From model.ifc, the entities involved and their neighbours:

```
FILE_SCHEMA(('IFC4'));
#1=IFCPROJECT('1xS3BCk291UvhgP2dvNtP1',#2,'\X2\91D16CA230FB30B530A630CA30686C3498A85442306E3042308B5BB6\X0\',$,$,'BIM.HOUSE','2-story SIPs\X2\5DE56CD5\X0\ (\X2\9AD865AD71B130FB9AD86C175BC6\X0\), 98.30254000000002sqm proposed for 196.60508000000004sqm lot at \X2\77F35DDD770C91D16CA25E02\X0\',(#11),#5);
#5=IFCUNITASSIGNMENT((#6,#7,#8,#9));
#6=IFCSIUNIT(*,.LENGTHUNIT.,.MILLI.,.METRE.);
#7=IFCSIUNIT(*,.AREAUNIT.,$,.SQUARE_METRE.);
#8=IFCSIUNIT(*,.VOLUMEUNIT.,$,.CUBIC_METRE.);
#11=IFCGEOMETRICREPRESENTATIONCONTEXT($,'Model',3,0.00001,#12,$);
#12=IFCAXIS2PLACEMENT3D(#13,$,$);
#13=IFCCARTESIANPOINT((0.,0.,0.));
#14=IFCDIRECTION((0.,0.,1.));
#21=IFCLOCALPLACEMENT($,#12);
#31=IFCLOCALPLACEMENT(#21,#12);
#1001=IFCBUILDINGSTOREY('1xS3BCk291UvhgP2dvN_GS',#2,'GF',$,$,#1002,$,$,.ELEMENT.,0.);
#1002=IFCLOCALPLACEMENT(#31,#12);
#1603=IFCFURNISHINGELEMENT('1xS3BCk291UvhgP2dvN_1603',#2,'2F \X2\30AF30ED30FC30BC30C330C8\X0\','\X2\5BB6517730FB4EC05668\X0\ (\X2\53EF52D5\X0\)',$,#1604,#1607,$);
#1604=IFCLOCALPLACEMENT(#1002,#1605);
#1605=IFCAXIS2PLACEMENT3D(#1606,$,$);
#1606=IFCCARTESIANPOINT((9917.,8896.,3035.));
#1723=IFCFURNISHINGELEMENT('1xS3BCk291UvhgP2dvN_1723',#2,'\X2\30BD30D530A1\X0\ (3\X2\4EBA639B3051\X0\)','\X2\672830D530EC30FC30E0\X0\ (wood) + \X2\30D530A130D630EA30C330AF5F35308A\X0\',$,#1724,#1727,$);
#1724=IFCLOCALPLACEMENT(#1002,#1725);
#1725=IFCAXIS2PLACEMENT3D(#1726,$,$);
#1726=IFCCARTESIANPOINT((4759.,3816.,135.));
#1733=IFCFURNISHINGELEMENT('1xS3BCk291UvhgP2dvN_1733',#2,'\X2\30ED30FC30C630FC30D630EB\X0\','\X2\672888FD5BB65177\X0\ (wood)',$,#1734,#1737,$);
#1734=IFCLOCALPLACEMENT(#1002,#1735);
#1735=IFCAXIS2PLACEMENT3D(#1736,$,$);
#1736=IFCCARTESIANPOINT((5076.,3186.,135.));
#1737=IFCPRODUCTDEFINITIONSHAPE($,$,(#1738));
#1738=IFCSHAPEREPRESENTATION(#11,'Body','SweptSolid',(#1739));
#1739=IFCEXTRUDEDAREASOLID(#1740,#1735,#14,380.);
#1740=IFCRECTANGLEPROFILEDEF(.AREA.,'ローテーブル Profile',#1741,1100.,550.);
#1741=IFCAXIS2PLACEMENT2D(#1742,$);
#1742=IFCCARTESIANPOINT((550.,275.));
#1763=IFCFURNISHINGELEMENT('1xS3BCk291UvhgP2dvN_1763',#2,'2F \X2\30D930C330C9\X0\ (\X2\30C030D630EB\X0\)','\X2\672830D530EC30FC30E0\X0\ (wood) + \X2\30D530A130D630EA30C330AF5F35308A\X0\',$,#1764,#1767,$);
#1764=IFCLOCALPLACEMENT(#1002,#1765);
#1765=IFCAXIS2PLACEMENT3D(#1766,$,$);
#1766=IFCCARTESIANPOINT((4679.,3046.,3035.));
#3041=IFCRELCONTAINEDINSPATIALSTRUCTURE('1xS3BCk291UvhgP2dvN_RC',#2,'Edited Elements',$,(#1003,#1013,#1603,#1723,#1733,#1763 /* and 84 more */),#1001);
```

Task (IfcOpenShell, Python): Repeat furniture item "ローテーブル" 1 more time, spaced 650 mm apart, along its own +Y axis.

```python
import ifcopenshell
import ifcopenshell.api.geometry
import ifcopenshell.api.root
import ifcopenshell.util.element
import ifcopenshell.util.placement
import ifcopenshell.util.unit

model = ifcopenshell.open("model.ifc")
unit_scale = ifcopenshell.util.unit.calculate_unit_scale(model)


def reuse_history(source, copy):
    """copy_class also copies each property set's owner history, people and application; keep the originals."""
    for rel in copy.IsDefinedBy:
        if rel.is_a("IfcRelDefinesByProperties") and (history := rel.RelatingPropertyDefinition.OwnerHistory):
            rel.RelatingPropertyDefinition.OwnerHistory = source.OwnerHistory
            ifcopenshell.util.element.remove_deep2(model, history)


source = model.by_guid("1xS3BCk291UvhgP2dvN_1733")
base = ifcopenshell.util.placement.get_local_placement(source.ObjectPlacement)
step = base[:3, 1] * 0.65 / unit_scale

for i in range(1, 2):
    copy = ifcopenshell.api.root.copy_class(model, product=source)
    copy.Representation = ifcopenshell.util.element.copy_deep(
        model, source.Representation, exclude=["IfcGeometricRepresentationContext", "IfcRepresentationMap"]
    )
    reuse_history(source, copy)
    matrix = base.copy()
    matrix[:3, 3] += i * step
    print("added at", matrix[:3, 3].round(3) + 0.0)
    ifcopenshell.api.geometry.edit_object_placement(model, product=copy, matrix=matrix, is_si=False)

model.write("model_edited.ifc")
```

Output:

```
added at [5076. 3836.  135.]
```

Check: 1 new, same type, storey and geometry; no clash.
